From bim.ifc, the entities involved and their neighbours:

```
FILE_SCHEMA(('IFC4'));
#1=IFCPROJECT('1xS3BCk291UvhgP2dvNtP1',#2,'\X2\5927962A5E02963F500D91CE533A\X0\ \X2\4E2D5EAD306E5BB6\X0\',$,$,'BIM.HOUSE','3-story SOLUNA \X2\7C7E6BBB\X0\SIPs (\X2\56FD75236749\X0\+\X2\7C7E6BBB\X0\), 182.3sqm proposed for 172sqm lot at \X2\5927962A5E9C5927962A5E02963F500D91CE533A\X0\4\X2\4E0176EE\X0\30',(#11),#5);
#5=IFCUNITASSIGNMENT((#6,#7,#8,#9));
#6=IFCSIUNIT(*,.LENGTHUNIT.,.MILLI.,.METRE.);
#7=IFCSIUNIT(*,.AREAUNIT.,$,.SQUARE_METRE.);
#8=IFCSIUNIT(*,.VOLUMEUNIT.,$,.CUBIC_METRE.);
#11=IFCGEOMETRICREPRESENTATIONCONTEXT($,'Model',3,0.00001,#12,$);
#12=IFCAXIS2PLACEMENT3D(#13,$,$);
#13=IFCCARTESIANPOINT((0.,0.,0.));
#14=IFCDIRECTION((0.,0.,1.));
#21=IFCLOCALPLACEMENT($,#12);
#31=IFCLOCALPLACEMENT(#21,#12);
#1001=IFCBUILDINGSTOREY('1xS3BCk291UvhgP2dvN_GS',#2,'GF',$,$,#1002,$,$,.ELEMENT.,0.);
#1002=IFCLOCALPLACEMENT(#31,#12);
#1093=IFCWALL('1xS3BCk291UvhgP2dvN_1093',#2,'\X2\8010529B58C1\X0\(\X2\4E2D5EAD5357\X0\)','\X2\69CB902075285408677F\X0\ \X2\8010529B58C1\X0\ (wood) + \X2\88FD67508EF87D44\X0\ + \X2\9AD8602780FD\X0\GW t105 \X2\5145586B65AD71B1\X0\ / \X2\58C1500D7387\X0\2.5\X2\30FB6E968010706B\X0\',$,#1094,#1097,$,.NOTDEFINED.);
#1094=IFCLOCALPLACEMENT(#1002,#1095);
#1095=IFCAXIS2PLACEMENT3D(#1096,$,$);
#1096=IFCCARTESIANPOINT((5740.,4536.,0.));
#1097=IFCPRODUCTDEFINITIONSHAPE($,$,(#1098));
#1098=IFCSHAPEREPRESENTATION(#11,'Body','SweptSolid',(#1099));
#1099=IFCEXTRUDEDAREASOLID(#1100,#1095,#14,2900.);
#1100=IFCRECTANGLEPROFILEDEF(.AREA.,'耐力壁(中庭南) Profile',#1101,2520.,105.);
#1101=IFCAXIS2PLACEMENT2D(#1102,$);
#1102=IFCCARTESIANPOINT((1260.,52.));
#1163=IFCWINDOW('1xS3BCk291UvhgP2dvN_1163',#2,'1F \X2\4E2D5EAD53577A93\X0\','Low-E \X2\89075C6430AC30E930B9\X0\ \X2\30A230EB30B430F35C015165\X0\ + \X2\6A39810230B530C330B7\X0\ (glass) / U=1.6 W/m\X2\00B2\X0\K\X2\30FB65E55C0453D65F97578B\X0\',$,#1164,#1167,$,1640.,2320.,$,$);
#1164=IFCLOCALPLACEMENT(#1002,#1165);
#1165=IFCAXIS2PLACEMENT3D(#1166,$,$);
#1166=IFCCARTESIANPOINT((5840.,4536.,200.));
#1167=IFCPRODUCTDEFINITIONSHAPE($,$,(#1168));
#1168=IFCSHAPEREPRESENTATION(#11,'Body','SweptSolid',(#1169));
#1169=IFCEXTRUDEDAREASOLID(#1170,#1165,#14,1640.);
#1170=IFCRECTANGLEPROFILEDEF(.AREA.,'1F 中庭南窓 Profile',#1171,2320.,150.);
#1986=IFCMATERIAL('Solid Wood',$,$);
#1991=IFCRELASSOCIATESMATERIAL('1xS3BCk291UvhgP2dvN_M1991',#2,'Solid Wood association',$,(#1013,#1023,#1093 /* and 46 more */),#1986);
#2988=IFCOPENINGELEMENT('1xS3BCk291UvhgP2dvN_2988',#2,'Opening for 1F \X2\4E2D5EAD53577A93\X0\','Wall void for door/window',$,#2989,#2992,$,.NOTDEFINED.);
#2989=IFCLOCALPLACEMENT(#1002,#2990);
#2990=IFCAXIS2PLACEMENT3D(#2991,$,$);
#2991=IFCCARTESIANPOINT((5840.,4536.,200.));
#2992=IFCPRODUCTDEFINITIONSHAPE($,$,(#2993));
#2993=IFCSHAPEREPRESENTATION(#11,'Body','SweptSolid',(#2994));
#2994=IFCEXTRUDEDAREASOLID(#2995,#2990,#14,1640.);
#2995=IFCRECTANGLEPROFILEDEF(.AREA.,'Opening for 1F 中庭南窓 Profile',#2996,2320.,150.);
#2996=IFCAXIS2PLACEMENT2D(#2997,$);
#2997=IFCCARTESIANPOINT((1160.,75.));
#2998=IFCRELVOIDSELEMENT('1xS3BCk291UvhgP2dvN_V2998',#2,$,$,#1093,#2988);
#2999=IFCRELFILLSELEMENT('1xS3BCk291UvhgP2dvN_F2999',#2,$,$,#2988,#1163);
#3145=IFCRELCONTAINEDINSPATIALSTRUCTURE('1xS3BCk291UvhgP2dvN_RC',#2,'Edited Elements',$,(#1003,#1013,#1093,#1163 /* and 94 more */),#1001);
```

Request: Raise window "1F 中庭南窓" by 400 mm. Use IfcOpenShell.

```python
import numpy as np
import ifcopenshell
import ifcopenshell.api.geometry
import ifcopenshell.util.placement
import ifcopenshell.util.unit

model = ifcopenshell.open("bim.ifc")
unit_scale = ifcopenshell.util.unit.calculate_unit_scale(model)

window = model.by_guid("1xS3BCk291UvhgP2dvN_1163")
opening = window.FillsVoids[0].RelatingOpeningElement
dz = 0.4 / unit_scale

shift = np.array([0.0, 0.0, dz])
# The window is not placed relative to its opening, so move both.
for product in (opening, window):
    matrix = ifcopenshell.util.placement.get_local_placement(product.ObjectPlacement)
    matrix[:3, 3] += shift
    ifcopenshell.api.geometry.edit_object_placement(model, product=product, matrix=matrix, is_si=False)

print(f"moved by {dz * unit_scale:+.3f} m")

model.write("bim_rev.ifc")
```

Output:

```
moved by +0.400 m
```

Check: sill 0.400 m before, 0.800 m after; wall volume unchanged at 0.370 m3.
